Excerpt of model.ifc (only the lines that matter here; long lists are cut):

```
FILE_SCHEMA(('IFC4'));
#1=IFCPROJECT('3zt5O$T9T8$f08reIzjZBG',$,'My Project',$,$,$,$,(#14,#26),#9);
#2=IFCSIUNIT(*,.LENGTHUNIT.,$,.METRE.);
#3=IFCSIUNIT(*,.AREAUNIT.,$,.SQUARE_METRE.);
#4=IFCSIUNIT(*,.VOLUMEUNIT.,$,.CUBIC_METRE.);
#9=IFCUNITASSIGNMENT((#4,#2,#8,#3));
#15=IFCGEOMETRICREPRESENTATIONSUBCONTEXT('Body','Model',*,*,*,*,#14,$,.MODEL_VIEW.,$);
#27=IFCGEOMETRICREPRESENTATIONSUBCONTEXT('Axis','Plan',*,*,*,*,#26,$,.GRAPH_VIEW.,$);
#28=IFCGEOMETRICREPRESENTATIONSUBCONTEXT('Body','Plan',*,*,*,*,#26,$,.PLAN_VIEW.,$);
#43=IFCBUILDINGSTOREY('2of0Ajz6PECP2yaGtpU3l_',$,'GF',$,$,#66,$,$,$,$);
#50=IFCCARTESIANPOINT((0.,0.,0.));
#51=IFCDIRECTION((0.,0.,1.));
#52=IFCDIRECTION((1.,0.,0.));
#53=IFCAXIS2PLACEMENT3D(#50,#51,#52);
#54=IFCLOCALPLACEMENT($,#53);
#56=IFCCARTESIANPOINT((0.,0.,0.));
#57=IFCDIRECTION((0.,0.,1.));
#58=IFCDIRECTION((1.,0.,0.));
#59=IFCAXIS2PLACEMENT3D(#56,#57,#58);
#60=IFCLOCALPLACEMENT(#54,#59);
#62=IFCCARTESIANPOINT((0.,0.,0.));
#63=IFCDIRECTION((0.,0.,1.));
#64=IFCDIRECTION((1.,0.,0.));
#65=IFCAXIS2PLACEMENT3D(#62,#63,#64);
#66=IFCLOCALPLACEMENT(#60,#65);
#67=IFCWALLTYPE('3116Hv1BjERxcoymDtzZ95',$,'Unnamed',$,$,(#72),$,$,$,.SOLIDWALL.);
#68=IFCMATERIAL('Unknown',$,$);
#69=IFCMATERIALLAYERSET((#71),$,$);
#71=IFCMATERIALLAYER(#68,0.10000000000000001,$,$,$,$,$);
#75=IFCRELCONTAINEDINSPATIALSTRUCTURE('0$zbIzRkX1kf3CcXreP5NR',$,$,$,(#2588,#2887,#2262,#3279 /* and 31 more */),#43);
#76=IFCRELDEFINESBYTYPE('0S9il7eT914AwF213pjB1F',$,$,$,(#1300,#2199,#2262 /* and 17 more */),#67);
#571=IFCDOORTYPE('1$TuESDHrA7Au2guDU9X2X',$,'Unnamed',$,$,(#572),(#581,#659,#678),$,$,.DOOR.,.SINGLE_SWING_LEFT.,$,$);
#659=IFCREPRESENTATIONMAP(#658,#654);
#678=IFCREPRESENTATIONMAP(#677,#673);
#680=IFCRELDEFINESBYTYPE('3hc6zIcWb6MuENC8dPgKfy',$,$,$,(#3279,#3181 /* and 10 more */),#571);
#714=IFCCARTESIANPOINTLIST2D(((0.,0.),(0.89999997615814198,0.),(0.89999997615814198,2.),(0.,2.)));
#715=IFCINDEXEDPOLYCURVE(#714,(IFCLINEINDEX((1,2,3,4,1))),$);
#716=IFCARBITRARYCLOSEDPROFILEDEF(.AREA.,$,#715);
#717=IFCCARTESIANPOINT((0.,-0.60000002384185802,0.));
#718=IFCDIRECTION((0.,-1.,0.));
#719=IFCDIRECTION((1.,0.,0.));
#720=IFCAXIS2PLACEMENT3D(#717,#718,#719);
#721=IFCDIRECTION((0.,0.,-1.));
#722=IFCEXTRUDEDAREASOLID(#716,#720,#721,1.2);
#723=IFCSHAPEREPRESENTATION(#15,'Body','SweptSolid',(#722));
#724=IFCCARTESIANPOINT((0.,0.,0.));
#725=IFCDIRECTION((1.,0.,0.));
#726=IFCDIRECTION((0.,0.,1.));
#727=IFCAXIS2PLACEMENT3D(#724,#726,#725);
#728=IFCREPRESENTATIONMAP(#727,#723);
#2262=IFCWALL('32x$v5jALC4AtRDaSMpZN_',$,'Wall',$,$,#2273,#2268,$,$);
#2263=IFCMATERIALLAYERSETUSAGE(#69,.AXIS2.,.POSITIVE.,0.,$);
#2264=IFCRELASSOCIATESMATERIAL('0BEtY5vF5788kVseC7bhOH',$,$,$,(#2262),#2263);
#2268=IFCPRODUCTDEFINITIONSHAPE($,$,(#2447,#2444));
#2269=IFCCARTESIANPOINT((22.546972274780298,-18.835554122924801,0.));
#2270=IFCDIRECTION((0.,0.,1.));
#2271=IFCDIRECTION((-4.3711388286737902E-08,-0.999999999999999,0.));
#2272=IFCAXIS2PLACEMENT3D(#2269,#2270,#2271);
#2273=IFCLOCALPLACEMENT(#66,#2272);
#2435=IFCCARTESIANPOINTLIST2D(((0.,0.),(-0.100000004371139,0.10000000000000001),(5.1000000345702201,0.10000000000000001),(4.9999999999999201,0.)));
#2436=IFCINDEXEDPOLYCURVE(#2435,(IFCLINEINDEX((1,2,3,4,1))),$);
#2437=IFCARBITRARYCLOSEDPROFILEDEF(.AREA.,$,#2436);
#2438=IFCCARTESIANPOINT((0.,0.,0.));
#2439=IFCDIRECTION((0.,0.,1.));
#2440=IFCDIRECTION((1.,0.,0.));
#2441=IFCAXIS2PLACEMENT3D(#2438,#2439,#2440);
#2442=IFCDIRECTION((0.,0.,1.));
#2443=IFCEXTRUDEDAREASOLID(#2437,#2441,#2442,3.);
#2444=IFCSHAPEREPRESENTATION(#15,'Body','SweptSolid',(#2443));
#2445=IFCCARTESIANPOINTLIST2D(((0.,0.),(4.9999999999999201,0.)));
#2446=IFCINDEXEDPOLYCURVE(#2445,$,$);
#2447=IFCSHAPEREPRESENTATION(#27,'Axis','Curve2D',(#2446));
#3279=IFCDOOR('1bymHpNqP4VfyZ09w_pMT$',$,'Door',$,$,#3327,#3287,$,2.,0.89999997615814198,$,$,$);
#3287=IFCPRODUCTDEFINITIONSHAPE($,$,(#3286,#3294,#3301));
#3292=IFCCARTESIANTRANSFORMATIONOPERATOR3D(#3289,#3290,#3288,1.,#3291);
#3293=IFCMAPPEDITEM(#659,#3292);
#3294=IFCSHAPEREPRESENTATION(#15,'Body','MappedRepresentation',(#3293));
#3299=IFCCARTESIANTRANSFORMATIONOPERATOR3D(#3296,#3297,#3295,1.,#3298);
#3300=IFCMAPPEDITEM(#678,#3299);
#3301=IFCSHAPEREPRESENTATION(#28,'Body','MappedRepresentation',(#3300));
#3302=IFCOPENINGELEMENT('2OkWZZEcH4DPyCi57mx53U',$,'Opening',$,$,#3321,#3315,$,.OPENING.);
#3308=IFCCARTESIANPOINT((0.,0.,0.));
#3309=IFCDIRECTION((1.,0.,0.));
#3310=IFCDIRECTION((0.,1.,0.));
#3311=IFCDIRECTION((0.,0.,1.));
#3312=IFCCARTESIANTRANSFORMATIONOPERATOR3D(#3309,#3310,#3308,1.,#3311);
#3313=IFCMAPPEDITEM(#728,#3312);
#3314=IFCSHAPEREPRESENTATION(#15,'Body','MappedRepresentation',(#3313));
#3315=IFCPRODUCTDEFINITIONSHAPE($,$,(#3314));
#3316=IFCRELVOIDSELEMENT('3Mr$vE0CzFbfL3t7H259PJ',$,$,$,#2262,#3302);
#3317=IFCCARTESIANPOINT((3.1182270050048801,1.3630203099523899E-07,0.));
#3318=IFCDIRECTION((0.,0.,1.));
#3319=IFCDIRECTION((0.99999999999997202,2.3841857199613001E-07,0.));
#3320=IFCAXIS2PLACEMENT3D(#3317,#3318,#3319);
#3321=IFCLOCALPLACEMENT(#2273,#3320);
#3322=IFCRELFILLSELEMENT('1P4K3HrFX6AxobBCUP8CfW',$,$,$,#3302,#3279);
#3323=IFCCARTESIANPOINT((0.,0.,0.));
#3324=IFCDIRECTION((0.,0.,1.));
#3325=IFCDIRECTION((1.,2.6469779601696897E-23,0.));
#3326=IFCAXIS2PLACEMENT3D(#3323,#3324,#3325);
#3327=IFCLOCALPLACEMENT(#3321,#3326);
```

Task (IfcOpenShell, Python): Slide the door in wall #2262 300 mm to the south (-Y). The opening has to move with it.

```python
import ifcopenshell
import ifcopenshell.api.geometry
import ifcopenshell.util.placement

model = ifcopenshell.open("model.ifc")

door = model.by_guid("1bymHpNqP4VfyZ09w_pMT$")
opening = door.FillsVoids[0].RelatingOpeningElement
wall = opening.VoidsElements[0].RelatingBuildingElement

wall_matrix = ifcopenshell.util.placement.get_local_placement(wall.ObjectPlacement)
shift = wall_matrix[:3, 0] * 0.3
before = ifcopenshell.util.placement.get_local_placement(door.ObjectPlacement)[:3, 3].copy()

# The door is placed relative to its opening, so it follows when the opening moves.
matrix = ifcopenshell.util.placement.get_local_placement(opening.ObjectPlacement)
matrix[:3, 3] += shift
ifcopenshell.api.geometry.edit_object_placement(
    model, product=opening, matrix=matrix, is_si=False, should_transform_children=True
)

after = ifcopenshell.util.placement.get_local_placement(door.ObjectPlacement)[:3, 3]
print("door moved by", (after - before).round(3) + 0.0)

model.write("model_rev.ifc")
```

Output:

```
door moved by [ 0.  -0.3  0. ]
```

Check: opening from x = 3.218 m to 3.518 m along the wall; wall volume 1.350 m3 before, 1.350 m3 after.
